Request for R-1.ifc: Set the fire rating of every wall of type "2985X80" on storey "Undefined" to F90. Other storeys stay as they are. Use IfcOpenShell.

First a look at what the model holds.

```python
import ifcopenshell
import ifcopenshell.util.element

model = ifcopenshell.open("R-1.ifc")
print(model.schema)
storey = next(s for s in model.by_type("IfcBuildingStorey") if s.Name == "Undefined")
walls = [e for e in ifcopenshell.util.element.get_decomposition(storey) if e.is_a("IfcWall")]
seen = {}
for e in walls:
    element_type = ifcopenshell.util.element.get_type(e)
    key = (element_type.Name if element_type != e and element_type else None, ifcopenshell.util.element.get_pset(e, "Pset_WallCommon", "FireRating"))
    seen[key] = seen.get(key, 0) + 1
for (name, value), count in sorted(seen.items(), key=str):
    print(count, "x", name, "|", value)
```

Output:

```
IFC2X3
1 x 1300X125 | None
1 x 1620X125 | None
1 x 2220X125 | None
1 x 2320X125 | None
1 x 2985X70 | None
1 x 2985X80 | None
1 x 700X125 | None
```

```python
import ifcopenshell
import ifcopenshell.api.pset
import ifcopenshell.util.element

model = ifcopenshell.open("R-1.ifc")

storey = next(s for s in model.by_type("IfcBuildingStorey") if s.Name == "Undefined")
walls = [e for e in ifcopenshell.util.element.get_decomposition(storey) if e.is_a("IfcWall")]

count = 0
for e in walls:
    element_type = ifcopenshell.util.element.get_type(e)
    if element_type in (None, e) or element_type.Name != "2985X80":
        continue
    # add_pset returns the element's existing set when there is one.
    pset = ifcopenshell.api.pset.add_pset(model, product=e, name="Pset_WallCommon")
    ifcopenshell.api.pset.edit_pset(model, pset=pset, properties={"FireRating": "F90"})
    count += 1

print(count, "walls updated")

model.write("R-1-out.ifc")
```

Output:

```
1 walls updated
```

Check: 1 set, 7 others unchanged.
